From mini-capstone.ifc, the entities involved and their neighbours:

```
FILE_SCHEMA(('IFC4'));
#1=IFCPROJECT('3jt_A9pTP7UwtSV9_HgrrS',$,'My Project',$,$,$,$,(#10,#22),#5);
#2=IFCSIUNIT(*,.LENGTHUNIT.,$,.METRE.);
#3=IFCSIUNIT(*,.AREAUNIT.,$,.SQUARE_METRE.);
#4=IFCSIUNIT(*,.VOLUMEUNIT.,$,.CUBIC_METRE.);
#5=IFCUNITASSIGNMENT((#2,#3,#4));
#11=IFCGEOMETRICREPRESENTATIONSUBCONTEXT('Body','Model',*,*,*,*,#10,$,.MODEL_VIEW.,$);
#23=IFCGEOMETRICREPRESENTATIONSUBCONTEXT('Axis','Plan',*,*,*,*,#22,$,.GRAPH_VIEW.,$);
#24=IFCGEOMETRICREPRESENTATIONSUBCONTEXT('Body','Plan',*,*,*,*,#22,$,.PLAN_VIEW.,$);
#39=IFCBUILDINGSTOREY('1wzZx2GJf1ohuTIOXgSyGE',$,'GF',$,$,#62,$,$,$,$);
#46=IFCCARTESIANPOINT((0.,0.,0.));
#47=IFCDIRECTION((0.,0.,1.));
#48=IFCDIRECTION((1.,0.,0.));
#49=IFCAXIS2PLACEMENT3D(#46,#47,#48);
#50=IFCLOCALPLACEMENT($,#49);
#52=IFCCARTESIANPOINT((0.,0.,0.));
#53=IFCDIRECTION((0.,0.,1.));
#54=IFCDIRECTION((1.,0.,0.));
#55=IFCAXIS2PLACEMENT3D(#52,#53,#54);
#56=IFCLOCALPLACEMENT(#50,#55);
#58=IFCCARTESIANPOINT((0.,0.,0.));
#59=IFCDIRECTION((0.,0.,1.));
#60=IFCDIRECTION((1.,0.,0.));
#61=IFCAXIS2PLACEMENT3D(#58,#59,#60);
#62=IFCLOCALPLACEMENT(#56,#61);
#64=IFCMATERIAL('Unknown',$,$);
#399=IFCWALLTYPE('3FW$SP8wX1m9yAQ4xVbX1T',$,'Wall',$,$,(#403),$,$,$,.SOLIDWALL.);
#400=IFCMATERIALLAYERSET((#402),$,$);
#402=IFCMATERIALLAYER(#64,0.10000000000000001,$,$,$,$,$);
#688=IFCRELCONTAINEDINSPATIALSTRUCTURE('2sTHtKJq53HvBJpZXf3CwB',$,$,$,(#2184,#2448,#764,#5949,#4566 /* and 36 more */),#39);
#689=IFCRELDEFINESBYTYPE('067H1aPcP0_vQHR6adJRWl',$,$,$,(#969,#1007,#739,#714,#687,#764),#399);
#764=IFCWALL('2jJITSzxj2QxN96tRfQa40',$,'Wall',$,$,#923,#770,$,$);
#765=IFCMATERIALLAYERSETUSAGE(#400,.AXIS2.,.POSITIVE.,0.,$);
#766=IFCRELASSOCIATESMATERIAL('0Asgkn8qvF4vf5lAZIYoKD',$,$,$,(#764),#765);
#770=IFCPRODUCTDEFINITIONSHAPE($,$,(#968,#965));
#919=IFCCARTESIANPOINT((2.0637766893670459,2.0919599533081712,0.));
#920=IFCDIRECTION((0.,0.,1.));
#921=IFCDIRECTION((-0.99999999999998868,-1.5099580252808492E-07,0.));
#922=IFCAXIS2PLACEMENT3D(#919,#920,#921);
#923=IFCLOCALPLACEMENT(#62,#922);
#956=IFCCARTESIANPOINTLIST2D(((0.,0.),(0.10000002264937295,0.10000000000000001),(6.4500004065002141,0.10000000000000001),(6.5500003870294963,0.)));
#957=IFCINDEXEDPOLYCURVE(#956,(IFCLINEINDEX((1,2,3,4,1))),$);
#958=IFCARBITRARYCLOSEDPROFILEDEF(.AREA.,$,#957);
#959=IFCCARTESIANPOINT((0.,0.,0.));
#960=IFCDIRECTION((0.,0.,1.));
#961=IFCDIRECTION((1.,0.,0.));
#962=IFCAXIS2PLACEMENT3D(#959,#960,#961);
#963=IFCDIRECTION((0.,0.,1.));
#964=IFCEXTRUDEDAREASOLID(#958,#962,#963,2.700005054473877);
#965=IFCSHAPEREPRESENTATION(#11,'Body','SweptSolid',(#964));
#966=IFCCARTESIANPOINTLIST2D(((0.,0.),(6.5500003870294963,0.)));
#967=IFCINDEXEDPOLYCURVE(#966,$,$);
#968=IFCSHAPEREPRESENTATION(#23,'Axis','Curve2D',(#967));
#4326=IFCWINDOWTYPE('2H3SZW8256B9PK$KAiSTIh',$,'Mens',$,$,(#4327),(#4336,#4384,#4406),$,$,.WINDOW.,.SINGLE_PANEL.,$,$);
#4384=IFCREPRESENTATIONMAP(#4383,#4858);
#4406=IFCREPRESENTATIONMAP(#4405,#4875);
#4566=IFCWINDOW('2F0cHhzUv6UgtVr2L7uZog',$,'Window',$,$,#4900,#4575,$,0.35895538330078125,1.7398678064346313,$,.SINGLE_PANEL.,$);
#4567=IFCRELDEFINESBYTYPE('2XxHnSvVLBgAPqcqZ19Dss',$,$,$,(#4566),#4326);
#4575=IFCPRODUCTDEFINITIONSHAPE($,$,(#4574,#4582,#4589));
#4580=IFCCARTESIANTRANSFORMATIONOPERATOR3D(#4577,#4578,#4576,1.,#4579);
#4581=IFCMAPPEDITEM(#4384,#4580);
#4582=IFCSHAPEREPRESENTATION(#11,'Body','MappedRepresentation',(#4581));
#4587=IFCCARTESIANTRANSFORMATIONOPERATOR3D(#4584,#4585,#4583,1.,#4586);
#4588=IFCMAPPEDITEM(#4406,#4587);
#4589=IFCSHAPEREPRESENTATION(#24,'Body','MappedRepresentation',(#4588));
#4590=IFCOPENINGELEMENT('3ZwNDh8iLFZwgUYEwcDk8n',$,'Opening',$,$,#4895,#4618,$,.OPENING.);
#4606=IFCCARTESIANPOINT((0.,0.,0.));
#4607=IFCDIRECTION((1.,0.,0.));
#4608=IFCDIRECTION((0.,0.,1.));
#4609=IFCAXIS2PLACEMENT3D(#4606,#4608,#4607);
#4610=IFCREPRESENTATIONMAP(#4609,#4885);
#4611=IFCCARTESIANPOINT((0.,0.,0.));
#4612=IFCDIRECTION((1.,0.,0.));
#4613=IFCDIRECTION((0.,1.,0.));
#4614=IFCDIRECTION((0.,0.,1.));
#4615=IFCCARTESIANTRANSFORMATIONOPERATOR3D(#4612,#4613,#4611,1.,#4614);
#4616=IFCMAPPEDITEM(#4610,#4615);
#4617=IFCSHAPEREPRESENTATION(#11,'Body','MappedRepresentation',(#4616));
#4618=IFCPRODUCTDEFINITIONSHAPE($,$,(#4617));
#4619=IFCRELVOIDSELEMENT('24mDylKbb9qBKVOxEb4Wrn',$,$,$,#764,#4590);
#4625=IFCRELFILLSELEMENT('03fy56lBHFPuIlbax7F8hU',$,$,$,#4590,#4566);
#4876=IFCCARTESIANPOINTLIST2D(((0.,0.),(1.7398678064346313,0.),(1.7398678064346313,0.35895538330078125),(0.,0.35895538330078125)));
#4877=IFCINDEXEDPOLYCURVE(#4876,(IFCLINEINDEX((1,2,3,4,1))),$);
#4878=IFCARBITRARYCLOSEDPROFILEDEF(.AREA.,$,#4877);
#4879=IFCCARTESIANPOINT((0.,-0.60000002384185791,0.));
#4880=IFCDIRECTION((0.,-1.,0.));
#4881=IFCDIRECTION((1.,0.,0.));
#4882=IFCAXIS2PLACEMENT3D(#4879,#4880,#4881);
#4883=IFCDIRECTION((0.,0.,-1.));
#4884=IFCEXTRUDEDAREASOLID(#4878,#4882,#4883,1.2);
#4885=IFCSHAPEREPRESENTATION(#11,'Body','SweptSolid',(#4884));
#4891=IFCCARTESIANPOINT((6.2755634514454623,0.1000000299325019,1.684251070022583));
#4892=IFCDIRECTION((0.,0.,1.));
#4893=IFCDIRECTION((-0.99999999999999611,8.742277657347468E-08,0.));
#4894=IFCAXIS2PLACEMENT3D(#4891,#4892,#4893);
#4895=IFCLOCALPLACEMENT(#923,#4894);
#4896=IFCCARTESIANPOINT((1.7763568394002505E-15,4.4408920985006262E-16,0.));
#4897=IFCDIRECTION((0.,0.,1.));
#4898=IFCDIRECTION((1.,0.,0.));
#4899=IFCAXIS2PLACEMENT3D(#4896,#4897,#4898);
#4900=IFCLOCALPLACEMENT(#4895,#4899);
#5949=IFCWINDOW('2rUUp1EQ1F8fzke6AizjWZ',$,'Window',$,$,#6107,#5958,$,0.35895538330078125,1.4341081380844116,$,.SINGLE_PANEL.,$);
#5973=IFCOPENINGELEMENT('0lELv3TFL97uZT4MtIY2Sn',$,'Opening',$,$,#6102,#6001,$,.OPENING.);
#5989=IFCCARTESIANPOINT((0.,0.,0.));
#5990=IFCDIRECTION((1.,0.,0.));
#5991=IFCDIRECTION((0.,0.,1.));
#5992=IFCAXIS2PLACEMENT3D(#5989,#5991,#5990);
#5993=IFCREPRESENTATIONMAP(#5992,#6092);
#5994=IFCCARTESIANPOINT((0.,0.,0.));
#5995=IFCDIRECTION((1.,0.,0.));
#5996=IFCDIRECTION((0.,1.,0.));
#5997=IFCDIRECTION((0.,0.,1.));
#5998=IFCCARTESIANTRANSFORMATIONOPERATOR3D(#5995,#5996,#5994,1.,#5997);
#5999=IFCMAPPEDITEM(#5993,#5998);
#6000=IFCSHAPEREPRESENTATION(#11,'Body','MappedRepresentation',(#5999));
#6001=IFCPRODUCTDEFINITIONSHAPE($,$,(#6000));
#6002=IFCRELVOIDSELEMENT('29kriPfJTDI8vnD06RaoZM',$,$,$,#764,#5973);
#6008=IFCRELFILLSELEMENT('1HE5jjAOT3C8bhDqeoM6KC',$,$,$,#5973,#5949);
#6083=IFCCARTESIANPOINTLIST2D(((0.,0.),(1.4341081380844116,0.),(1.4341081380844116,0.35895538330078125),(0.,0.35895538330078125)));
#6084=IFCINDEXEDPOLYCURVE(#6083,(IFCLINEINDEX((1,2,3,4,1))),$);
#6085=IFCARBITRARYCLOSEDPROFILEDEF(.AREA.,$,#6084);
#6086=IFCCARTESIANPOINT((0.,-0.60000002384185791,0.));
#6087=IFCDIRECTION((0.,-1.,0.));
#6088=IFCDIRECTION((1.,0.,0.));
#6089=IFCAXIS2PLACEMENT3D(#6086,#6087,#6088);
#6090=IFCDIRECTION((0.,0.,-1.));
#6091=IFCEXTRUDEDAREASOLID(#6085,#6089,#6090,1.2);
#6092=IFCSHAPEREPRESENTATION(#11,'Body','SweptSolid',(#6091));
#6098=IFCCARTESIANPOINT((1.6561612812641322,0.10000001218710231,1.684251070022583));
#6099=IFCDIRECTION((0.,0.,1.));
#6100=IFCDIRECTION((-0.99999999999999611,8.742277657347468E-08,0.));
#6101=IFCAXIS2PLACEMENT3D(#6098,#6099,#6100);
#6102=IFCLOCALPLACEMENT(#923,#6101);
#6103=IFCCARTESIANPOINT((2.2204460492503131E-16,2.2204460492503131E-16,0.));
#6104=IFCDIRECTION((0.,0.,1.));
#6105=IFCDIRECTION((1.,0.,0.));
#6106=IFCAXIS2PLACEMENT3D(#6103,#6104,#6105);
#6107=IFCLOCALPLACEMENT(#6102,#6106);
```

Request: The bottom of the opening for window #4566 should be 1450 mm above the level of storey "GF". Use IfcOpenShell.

```python
import numpy as np
import ifcopenshell
import ifcopenshell.api.geometry
import ifcopenshell.geom
import ifcopenshell.util.element
import ifcopenshell.util.placement
import ifcopenshell.util.shape
import ifcopenshell.util.unit

model = ifcopenshell.open("mini-capstone.ifc")
unit_scale = ifcopenshell.util.unit.calculate_unit_scale(model)

window = model.by_guid("2F0cHhzUv6UgtVr2L7uZog")
opening = window.FillsVoids[0].RelatingOpeningElement
storey = ifcopenshell.util.element.get_container(window, ifc_class="IfcBuildingStorey")
level = ifcopenshell.util.placement.get_local_placement(storey.ObjectPlacement)[2, 3]

# The opening's origin need not be at the sill, so measure its lowest point.
shape = ifcopenshell.geom.create_shape(ifcopenshell.geom.settings(), opening)
bottom = ifcopenshell.util.shape.get_shape_bottom_elevation(shape, shape.geometry) / unit_scale
dz = level + 1.45 - bottom

shift = np.array([0.0, 0.0, dz])
# The window is placed relative to its opening, so it follows when the opening moves.
matrix = ifcopenshell.util.placement.get_local_placement(opening.ObjectPlacement)
matrix[:3, 3] += shift
ifcopenshell.api.geometry.edit_object_placement(
    model, product=opening, matrix=matrix, is_si=False, should_transform_children=True
)

print(f"moved by {dz * unit_scale:+.3f} m")

model.write("mini-capstone_updated.ifc")
```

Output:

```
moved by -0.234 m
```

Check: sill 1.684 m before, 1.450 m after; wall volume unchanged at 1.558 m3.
